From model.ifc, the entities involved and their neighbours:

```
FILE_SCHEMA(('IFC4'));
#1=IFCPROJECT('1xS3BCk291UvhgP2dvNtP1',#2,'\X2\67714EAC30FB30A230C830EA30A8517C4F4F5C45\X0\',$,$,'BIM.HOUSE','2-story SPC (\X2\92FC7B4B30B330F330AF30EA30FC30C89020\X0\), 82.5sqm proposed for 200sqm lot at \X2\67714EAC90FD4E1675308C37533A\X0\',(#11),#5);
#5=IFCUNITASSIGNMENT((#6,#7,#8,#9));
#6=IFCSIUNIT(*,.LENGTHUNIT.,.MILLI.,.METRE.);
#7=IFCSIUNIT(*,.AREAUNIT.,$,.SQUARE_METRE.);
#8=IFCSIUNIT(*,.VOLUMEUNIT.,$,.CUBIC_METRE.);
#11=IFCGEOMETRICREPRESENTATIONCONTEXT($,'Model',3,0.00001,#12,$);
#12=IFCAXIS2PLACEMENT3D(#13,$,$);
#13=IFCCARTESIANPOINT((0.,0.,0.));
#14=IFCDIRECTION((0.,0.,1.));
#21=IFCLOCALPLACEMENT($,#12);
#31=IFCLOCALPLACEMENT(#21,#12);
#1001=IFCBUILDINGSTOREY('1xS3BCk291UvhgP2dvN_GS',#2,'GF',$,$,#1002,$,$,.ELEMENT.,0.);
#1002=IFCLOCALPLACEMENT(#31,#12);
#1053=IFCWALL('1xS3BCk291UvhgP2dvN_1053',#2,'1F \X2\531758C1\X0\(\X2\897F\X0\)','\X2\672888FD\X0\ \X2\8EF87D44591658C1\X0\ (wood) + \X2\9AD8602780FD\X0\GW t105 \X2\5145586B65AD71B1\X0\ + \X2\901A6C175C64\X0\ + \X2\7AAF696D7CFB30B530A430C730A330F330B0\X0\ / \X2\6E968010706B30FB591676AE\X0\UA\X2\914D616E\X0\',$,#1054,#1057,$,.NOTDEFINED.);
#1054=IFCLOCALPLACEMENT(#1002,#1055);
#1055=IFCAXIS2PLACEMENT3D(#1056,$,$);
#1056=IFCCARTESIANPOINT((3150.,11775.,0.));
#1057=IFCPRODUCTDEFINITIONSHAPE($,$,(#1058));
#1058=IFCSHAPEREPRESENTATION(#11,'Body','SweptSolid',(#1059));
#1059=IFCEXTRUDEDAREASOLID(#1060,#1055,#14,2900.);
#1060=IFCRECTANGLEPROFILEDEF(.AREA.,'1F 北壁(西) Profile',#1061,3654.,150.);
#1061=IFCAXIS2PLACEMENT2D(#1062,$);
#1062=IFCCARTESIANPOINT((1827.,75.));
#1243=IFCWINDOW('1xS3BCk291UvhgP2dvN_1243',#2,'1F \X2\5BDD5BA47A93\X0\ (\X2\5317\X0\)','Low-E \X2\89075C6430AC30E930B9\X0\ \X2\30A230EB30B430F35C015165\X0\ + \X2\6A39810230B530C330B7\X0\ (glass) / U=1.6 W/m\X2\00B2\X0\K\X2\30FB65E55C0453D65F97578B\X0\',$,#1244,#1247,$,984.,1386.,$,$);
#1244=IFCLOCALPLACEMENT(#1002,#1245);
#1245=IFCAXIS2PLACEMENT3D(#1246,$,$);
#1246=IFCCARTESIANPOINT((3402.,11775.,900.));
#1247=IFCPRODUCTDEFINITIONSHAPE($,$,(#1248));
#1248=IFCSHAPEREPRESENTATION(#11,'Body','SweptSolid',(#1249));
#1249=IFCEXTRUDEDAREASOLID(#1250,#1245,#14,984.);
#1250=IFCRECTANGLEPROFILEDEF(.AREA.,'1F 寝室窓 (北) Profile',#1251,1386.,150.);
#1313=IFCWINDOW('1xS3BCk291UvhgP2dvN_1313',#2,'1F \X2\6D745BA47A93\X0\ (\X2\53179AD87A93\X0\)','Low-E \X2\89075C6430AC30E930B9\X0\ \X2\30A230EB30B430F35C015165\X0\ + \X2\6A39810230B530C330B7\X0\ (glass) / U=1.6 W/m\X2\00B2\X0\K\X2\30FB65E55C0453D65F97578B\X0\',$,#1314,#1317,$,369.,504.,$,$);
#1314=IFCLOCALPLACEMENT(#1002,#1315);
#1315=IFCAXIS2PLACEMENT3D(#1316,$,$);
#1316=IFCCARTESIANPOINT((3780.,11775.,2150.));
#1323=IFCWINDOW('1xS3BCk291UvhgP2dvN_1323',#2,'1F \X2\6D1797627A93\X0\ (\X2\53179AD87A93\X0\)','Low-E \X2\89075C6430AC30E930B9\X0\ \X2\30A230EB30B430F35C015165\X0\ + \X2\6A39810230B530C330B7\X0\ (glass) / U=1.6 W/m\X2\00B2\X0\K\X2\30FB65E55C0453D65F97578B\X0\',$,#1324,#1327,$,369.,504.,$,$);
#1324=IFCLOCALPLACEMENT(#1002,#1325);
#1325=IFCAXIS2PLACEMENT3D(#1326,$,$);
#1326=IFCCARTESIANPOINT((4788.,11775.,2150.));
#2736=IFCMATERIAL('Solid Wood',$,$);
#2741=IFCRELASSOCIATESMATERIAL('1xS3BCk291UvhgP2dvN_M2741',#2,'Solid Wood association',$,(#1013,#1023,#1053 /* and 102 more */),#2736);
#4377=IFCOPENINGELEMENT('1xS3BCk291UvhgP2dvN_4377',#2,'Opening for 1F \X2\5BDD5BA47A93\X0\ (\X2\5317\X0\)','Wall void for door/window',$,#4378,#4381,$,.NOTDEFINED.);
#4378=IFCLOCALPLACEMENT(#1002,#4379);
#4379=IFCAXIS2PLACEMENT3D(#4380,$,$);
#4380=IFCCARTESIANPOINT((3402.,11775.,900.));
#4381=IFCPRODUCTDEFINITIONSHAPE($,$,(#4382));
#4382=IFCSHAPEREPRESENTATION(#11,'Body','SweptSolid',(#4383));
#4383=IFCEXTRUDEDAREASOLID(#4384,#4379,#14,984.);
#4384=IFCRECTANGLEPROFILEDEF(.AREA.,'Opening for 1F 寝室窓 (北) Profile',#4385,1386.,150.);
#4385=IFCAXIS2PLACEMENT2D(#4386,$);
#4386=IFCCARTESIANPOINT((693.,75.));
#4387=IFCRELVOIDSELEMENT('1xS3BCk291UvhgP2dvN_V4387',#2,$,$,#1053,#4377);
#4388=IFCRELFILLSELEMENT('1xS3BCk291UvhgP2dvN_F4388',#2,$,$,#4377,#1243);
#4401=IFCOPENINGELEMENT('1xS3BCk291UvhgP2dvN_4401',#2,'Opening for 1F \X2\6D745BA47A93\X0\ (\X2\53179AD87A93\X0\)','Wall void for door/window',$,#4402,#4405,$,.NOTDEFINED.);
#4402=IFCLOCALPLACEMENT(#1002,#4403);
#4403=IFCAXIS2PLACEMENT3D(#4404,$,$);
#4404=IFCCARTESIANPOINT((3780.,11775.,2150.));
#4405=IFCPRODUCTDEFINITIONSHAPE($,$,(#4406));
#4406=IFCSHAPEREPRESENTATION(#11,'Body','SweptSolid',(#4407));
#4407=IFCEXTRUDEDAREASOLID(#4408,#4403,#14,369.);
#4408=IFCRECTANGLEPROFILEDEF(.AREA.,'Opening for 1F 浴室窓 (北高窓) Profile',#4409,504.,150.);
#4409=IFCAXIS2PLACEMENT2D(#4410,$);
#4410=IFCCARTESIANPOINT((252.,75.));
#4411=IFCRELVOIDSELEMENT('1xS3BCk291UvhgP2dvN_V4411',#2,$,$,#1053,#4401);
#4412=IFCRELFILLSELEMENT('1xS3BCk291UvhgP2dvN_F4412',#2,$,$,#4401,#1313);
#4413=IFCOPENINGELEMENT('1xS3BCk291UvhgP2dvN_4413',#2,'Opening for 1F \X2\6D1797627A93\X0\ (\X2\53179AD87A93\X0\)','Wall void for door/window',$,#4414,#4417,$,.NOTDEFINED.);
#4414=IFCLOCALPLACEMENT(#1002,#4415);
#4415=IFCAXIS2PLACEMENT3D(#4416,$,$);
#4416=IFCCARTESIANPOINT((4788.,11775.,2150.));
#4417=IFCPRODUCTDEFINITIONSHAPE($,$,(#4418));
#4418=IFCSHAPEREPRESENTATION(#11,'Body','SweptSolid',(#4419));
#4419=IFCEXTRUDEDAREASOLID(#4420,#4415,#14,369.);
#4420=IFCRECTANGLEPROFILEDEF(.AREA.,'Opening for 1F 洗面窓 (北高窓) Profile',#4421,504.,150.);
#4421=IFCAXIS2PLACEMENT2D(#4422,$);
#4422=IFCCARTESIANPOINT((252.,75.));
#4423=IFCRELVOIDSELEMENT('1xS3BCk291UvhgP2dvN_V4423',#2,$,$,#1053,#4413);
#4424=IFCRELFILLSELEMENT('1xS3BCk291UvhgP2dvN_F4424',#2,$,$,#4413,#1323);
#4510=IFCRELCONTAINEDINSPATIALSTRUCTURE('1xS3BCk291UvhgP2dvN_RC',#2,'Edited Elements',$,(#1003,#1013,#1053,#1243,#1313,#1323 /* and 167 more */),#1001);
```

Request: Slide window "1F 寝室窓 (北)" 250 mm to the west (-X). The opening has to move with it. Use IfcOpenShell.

```python
import ifcopenshell
import ifcopenshell.api.geometry
import ifcopenshell.util.placement
import ifcopenshell.util.unit

model = ifcopenshell.open("model.ifc")
unit_scale = ifcopenshell.util.unit.calculate_unit_scale(model)

window = model.by_guid("1xS3BCk291UvhgP2dvN_1243")
opening = window.FillsVoids[0].RelatingOpeningElement
wall = opening.VoidsElements[0].RelatingBuildingElement

wall_matrix = ifcopenshell.util.placement.get_local_placement(wall.ObjectPlacement)
shift = wall_matrix[:3, 0] * -0.25 / unit_scale
before = ifcopenshell.util.placement.get_local_placement(window.ObjectPlacement)[:3, 3].copy()

# The window is not placed relative to its opening, so move both.
for product in (opening, window):
    matrix = ifcopenshell.util.placement.get_local_placement(product.ObjectPlacement)
    matrix[:3, 3] += shift
    ifcopenshell.api.geometry.edit_object_placement(model, product=product, matrix=matrix, is_si=False)

after = ifcopenshell.util.placement.get_local_placement(window.ObjectPlacement)[:3, 3]
print("window moved by", (after - before).round(3) + 0.0)

model.write("model_edited.ifc")
```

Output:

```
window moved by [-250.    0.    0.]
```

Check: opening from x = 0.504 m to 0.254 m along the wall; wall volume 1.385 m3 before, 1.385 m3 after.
